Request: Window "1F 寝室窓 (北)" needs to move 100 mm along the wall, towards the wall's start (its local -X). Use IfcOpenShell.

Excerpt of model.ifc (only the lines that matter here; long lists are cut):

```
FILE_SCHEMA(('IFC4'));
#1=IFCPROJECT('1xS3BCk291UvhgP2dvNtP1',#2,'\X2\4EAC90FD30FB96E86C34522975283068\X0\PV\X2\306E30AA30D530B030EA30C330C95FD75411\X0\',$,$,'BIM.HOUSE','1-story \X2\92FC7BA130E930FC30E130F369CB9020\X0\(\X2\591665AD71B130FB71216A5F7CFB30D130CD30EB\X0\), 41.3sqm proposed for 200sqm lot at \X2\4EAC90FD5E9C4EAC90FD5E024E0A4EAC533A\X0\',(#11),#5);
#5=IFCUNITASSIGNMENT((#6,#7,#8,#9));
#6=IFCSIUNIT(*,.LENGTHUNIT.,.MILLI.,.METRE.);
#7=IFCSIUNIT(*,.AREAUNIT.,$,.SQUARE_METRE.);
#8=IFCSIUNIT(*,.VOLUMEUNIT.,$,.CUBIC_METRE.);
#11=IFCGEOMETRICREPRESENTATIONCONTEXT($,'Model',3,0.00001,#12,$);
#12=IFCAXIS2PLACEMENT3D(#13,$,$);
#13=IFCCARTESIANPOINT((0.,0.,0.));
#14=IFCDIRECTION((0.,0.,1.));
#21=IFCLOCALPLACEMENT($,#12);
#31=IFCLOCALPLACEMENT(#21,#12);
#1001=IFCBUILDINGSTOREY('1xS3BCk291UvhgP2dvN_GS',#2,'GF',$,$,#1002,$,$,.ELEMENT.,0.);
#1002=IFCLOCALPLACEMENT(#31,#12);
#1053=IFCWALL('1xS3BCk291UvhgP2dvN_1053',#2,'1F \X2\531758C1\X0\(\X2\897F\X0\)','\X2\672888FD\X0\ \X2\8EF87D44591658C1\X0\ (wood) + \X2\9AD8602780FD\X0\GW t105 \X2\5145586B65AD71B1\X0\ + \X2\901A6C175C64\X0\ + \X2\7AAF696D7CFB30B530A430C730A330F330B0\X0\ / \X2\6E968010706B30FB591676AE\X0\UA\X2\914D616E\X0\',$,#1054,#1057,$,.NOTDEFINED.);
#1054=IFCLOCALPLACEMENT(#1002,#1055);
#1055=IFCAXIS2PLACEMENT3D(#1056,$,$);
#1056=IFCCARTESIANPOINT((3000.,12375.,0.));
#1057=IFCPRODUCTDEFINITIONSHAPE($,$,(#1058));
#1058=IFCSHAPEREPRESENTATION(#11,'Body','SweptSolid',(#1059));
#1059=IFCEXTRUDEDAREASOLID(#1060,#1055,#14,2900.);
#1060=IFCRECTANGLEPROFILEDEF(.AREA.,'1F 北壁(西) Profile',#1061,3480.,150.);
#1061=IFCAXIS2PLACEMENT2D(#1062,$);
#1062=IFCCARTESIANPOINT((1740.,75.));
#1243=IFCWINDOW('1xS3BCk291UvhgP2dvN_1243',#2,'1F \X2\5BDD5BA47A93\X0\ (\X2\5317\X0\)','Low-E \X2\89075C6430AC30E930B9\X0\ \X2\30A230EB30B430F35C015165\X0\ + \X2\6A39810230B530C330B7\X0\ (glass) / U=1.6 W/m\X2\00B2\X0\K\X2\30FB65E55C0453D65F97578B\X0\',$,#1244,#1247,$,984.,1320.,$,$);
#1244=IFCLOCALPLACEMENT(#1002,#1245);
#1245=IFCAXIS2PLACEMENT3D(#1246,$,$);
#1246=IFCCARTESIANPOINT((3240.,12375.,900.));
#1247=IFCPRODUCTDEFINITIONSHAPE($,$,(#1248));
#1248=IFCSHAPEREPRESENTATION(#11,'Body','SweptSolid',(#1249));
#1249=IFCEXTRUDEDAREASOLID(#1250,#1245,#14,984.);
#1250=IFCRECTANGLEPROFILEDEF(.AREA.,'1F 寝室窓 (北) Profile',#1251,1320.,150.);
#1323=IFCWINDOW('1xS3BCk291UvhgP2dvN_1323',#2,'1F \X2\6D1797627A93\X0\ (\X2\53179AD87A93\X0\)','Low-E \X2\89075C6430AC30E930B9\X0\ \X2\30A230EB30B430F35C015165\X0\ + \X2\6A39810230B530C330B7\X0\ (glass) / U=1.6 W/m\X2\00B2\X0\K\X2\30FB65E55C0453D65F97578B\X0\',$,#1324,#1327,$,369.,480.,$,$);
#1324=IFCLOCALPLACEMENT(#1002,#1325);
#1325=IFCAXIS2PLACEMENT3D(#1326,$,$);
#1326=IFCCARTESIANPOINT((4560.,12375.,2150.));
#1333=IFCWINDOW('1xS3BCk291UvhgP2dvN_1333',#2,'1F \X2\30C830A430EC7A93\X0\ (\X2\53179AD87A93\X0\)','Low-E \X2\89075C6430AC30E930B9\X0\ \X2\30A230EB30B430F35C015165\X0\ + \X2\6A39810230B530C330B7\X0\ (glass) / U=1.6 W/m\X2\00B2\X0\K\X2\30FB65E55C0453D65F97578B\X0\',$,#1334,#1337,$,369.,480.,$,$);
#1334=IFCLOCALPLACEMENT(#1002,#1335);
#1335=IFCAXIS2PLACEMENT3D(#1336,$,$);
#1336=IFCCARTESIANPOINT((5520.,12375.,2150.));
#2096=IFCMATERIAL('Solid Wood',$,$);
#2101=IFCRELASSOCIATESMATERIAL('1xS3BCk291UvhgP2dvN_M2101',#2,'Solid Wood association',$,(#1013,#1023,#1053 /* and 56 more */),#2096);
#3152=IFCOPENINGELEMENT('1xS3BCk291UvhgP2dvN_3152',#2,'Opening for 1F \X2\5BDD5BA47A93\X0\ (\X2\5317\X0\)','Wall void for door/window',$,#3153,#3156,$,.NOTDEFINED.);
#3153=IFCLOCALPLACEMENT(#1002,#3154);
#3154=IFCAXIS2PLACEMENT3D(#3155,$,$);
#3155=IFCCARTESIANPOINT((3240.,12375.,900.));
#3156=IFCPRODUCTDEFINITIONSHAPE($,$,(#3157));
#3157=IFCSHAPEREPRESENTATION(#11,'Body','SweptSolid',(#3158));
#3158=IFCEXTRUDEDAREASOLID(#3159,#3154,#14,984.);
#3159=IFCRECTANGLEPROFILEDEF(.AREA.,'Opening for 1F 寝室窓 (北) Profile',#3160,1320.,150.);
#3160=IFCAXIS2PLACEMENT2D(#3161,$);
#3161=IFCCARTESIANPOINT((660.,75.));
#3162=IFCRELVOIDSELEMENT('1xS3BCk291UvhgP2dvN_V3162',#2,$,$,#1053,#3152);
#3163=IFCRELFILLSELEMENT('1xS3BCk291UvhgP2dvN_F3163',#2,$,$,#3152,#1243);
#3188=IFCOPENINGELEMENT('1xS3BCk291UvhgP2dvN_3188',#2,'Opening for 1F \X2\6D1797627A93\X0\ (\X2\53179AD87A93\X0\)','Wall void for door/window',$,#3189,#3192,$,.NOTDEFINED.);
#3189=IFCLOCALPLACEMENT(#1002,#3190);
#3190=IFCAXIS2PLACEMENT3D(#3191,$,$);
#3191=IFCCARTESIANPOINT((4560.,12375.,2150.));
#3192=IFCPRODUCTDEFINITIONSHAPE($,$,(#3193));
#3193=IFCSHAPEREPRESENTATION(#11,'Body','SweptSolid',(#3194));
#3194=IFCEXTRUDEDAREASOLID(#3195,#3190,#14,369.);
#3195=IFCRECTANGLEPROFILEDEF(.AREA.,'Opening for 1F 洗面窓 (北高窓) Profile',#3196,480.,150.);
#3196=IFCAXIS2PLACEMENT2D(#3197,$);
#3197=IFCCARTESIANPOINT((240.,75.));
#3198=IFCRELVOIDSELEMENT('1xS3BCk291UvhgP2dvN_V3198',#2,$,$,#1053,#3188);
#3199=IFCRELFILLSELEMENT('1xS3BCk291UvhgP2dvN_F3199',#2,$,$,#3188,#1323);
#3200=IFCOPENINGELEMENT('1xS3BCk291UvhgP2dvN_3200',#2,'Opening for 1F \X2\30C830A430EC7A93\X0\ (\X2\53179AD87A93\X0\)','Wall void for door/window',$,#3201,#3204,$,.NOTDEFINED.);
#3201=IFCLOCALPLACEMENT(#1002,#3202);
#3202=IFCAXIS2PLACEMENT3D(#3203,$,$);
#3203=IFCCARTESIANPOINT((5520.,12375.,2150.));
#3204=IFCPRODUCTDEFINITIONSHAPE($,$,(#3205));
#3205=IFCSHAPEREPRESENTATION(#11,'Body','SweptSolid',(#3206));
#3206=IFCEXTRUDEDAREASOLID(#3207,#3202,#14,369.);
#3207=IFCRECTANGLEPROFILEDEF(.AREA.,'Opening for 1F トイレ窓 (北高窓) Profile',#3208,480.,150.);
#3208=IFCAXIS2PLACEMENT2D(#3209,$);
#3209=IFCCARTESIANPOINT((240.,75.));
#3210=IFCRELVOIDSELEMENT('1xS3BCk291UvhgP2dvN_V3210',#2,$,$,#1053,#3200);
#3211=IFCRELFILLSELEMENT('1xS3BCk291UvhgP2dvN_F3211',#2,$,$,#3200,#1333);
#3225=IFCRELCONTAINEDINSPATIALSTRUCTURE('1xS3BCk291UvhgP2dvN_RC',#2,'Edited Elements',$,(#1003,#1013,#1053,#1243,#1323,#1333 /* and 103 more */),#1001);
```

```python
import ifcopenshell
import ifcopenshell.api.geometry
import ifcopenshell.util.placement

model = ifcopenshell.open("model.ifc")

window = model.by_guid("1xS3BCk291UvhgP2dvN_1243")
opening = window.FillsVoids[0].RelatingOpeningElement
wall = opening.VoidsElements[0].RelatingBuildingElement

wall_matrix = ifcopenshell.util.placement.get_local_placement(wall.ObjectPlacement)
shift = wall_matrix[:3, 0] * -100.0
before = ifcopenshell.util.placement.get_local_placement(window.ObjectPlacement)[:3, 3].copy()

# The window is not placed relative to its opening, so move both.
for product in (opening, window):
    matrix = ifcopenshell.util.placement.get_local_placement(product.ObjectPlacement)
    matrix[:3, 3] += shift
    ifcopenshell.api.geometry.edit_object_placement(model, product=product, matrix=matrix, is_si=False)

after = ifcopenshell.util.placement.get_local_placement(window.ObjectPlacement)[:3, 3]
print("window moved by", (after - before).round(3) + 0.0)

model.write("model-out.ifc")
```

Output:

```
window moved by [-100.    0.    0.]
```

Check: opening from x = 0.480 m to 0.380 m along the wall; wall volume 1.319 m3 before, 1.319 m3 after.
